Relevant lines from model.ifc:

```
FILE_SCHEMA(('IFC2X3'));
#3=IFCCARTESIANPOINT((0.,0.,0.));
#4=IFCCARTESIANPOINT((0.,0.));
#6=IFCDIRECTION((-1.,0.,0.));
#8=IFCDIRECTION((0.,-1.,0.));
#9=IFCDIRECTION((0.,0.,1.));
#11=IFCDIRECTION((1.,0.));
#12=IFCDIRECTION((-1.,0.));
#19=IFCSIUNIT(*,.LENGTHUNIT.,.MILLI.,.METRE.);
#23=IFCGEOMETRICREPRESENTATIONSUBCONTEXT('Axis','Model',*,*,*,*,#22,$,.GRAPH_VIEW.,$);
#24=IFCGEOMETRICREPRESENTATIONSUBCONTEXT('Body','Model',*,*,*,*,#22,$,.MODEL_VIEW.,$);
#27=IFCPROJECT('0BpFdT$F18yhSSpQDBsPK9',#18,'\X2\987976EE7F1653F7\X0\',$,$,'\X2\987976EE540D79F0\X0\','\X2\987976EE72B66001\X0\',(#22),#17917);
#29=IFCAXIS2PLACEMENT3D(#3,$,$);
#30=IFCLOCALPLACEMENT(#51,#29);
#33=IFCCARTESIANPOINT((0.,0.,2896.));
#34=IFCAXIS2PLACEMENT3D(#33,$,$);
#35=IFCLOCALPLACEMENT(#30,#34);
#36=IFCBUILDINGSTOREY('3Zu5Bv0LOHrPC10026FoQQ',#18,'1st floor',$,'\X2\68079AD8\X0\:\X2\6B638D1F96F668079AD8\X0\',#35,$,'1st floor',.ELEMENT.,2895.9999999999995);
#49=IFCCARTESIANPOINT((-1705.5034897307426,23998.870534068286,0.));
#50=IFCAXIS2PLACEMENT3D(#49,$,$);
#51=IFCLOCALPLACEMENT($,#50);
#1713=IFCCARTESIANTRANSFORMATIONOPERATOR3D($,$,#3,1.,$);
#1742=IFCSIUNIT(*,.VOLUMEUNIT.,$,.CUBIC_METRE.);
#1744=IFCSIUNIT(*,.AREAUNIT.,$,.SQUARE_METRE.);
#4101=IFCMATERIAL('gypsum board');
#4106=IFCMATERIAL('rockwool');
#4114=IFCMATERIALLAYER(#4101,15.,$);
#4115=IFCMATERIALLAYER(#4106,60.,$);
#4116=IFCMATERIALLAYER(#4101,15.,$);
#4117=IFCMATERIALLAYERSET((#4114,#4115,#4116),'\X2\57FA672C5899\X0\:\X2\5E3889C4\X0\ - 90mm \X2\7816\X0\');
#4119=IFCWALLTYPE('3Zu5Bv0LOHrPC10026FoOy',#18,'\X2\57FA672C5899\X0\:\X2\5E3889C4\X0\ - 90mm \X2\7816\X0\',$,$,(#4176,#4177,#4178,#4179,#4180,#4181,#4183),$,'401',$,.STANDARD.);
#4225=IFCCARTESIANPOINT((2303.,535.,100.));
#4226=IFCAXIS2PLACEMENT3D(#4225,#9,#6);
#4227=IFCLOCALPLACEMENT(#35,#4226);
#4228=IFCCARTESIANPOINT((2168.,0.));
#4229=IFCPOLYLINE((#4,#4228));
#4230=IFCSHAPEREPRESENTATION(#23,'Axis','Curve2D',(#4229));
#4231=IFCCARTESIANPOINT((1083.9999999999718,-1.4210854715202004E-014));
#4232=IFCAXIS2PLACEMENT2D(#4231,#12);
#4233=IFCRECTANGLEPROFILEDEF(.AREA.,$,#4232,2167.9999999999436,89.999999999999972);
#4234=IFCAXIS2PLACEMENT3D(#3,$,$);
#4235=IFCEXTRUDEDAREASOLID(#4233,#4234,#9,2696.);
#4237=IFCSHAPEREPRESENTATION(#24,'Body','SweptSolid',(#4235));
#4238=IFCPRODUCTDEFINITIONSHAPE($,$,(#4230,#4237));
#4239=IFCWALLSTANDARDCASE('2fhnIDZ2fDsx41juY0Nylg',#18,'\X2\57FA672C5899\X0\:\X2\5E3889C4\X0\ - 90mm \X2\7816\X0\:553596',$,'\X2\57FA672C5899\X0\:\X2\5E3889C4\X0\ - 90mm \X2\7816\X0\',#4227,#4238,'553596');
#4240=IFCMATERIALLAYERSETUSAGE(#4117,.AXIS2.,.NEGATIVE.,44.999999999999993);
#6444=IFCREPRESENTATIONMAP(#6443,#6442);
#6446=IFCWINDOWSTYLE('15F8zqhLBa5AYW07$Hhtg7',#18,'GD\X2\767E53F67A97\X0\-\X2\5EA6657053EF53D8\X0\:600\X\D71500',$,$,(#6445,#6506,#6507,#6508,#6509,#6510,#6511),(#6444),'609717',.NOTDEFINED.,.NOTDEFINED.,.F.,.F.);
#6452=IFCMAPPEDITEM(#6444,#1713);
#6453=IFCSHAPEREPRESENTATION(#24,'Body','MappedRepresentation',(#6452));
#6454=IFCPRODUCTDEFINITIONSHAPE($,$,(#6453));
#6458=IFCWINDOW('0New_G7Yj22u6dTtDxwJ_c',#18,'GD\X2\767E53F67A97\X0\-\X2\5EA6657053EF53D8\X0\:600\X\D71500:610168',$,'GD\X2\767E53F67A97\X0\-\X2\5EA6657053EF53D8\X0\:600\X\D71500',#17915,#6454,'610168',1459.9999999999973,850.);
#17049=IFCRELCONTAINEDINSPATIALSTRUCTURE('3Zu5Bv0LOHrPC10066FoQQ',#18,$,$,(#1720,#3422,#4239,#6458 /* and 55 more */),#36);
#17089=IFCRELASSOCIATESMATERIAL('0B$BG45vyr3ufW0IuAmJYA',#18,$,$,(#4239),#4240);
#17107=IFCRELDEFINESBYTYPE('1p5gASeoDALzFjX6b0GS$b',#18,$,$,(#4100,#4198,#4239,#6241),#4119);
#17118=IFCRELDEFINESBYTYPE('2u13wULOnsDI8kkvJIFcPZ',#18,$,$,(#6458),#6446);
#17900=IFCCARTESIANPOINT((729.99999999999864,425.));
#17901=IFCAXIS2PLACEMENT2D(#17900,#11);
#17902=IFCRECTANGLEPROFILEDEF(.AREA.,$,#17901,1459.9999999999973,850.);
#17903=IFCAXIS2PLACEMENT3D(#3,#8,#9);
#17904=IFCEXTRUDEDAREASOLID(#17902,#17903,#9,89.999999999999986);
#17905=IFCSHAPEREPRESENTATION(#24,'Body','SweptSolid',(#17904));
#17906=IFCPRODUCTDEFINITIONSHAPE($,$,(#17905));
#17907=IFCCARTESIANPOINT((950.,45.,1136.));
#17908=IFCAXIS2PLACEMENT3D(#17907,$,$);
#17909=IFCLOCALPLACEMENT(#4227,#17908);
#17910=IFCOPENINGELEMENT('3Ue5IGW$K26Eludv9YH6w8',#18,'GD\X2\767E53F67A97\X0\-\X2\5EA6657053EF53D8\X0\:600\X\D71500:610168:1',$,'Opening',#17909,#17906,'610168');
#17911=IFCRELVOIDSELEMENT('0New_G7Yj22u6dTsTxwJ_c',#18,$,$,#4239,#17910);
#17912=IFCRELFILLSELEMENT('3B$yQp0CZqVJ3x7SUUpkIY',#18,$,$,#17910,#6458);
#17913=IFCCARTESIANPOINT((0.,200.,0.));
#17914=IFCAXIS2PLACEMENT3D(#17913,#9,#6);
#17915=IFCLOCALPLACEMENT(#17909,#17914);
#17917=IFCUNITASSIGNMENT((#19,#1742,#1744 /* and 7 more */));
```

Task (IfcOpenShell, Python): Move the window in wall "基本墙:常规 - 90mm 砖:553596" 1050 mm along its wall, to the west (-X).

```python
import ifcopenshell
import ifcopenshell.api.geometry
import ifcopenshell.util.placement
import ifcopenshell.util.unit

model = ifcopenshell.open("model.ifc")
unit_scale = ifcopenshell.util.unit.calculate_unit_scale(model)

window = model.by_guid("0New_G7Yj22u6dTtDxwJ_c")
opening = window.FillsVoids[0].RelatingOpeningElement
wall = opening.VoidsElements[0].RelatingBuildingElement

wall_matrix = ifcopenshell.util.placement.get_local_placement(wall.ObjectPlacement)
shift = wall_matrix[:3, 0] * 1.05 / unit_scale
before = ifcopenshell.util.placement.get_local_placement(window.ObjectPlacement)[:3, 3].copy()

# The window is placed relative to its opening, so it follows when the opening moves.
matrix = ifcopenshell.util.placement.get_local_placement(opening.ObjectPlacement)
matrix[:3, 3] += shift
ifcopenshell.api.geometry.edit_object_placement(
    model, product=opening, matrix=matrix, is_si=False, should_transform_children=True
)

after = ifcopenshell.util.placement.get_local_placement(window.ObjectPlacement)[:3, 3]
print("window moved by", (after - before).round(3) + 0.0)

model.write("model_edited.ifc")
```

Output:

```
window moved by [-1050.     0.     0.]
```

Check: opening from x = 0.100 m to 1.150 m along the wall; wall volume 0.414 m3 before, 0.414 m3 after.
